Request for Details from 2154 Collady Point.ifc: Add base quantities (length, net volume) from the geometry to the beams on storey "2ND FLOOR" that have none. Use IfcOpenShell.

First a look at what the model holds.

```python
import ifcopenshell
import ifcopenshell.util.element
import ifcopenshell.util.unit

model = ifcopenshell.open("Details from 2154 Collady Point.ifc")
print(model.schema)
for unit_type in ("LENGTHUNIT", "AREAUNIT", "VOLUMEUNIT"):
    print(unit_type, ifcopenshell.util.unit.calculate_unit_scale(model, unit_type))
storey = next(s for s in model.by_type("IfcBuildingStorey") if s.Name == "2ND FLOOR")
beams = [e for e in ifcopenshell.util.element.get_decomposition(storey) if e.is_a("IfcBeam")]
for e in sorted(beams, key=lambda e: e.id()):
    print(e.id(), e.is_a(), e.Name, list(ifcopenshell.util.element.get_psets(e, qtos_only=True)), sep=" | ")
```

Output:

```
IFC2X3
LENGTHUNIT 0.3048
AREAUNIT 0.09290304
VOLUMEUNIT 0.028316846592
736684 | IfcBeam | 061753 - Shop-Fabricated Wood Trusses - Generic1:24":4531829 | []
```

```python
import ifcopenshell
import ifcopenshell.api.pset
import ifcopenshell.geom
import ifcopenshell.util.element
import ifcopenshell.util.shape
import ifcopenshell.util.unit

model = ifcopenshell.open("Details from 2154 Collady Point.ifc")
unit_scale = ifcopenshell.util.unit.calculate_unit_scale(model)
volume_scale = ifcopenshell.util.unit.calculate_unit_scale(model, "VOLUMEUNIT")
settings = ifcopenshell.geom.settings()

storey = next(s for s in model.by_type("IfcBuildingStorey") if s.Name == "2ND FLOOR")
beams = [e for e in ifcopenshell.util.element.get_decomposition(storey) if e.is_a("IfcBeam")]

for e in sorted(beams, key=lambda e: e.id()):
    if ifcopenshell.util.element.get_psets(e, qtos_only=True, should_inherit=False):
        continue
    # Geometry comes back in metres, in the element's own axes.
    shape = ifcopenshell.geom.create_shape(settings, e)
    values = {
        "Length": ifcopenshell.util.shape.get_max_xyz(shape.geometry) / unit_scale,
        "NetVolume": ifcopenshell.util.shape.get_volume(shape.geometry) / volume_scale,
    }
    qto = ifcopenshell.api.pset.add_qto(model, product=e, name="BaseQuantities")
    ifcopenshell.api.pset.edit_qto(model, qto=qto, properties=values)
    print(e.id(), {k: round(v, 3) for k, v in values.items()})

model.write("Details from 2154 Collady Point_v2.ifc")
```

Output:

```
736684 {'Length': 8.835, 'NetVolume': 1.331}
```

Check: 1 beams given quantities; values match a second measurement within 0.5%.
